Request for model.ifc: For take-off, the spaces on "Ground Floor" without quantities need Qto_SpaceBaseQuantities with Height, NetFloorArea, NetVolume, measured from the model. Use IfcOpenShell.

First a look at what the model holds.

```python
import ifcopenshell
import ifcopenshell.util.element
import ifcopenshell.util.unit

model = ifcopenshell.open("model.ifc")
print(model.schema)
for unit_type in ("LENGTHUNIT", "AREAUNIT", "VOLUMEUNIT"):
    print(unit_type, ifcopenshell.util.unit.calculate_unit_scale(model, unit_type))
storey = next(s for s in model.by_type("IfcBuildingStorey") if s.Name == "Ground Floor")
spaces = [e for e in ifcopenshell.util.element.get_decomposition(storey) if e.is_a("IfcSpace")]
for e in sorted(spaces, key=lambda e: e.id()):
    print(e.id(), e.is_a(), e.Name, list(ifcopenshell.util.element.get_psets(e, qtos_only=True)), sep=" | ")
```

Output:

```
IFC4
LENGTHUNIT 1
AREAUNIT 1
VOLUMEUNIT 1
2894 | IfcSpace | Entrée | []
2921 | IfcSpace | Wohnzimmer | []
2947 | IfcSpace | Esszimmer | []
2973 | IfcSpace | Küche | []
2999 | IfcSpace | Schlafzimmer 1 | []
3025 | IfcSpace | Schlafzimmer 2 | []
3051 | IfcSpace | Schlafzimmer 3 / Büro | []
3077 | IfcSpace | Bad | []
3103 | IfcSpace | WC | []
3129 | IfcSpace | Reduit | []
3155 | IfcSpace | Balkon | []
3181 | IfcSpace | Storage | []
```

```python
import ifcopenshell
import ifcopenshell.api.pset
import ifcopenshell.geom
import ifcopenshell.util.element
import ifcopenshell.util.shape
import ifcopenshell.util.unit

model = ifcopenshell.open("model.ifc")
unit_scale = ifcopenshell.util.unit.calculate_unit_scale(model)
area_scale = ifcopenshell.util.unit.calculate_unit_scale(model, "AREAUNIT")
volume_scale = ifcopenshell.util.unit.calculate_unit_scale(model, "VOLUMEUNIT")
settings = ifcopenshell.geom.settings()

storey = next(s for s in model.by_type("IfcBuildingStorey") if s.Name == "Ground Floor")
spaces = [e for e in ifcopenshell.util.element.get_decomposition(storey) if e.is_a("IfcSpace")]

for e in sorted(spaces, key=lambda e: e.id()):
    if ifcopenshell.util.element.get_psets(e, qtos_only=True, should_inherit=False):
        continue
    # Geometry comes back in metres, in the element's own axes.
    shape = ifcopenshell.geom.create_shape(settings, e)
    values = {
        "Height": ifcopenshell.util.shape.get_z(shape.geometry) / unit_scale,
        "NetFloorArea": ifcopenshell.util.shape.get_footprint_area(shape.geometry) / area_scale,
        "NetVolume": ifcopenshell.util.shape.get_volume(shape.geometry) / volume_scale,
    }
    qto = ifcopenshell.api.pset.add_qto(model, product=e, name="Qto_SpaceBaseQuantities")
    ifcopenshell.api.pset.edit_qto(model, qto=qto, properties=values)
    print(e.id(), {k: round(v, 3) for k, v in values.items()})

model.write("model-out.ifc")
```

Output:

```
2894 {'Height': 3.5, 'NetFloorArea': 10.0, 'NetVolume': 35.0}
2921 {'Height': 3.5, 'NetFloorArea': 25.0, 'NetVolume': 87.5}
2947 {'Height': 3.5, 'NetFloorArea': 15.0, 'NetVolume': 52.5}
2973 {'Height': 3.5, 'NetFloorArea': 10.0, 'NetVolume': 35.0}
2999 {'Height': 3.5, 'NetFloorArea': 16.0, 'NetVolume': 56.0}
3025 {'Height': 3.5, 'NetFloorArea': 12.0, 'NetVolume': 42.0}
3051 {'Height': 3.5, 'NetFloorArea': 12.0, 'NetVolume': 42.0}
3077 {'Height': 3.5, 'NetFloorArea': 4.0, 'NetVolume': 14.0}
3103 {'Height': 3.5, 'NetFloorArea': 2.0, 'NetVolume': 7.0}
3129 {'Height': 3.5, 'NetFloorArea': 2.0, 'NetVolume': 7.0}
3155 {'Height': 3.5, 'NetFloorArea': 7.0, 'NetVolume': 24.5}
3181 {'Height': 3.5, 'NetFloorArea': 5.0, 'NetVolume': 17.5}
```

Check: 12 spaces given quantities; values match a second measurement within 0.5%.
